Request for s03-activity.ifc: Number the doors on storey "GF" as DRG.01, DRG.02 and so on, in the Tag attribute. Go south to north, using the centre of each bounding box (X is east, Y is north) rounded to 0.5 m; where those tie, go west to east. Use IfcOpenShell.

First a look at what the model holds.

```python
import ifcopenshell
import ifcopenshell.util.element
import ifcopenshell.util.placement

model = ifcopenshell.open("s03-activity.ifc")
print(model.schema)
storey = next(s for s in model.by_type("IfcBuildingStorey") if s.Name == "GF")
doors = [e for e in ifcopenshell.util.element.get_decomposition(storey) if e.is_a("IfcDoor")]
for e in sorted(doors, key=lambda e: e.id()):
    origin = ifcopenshell.util.placement.get_local_placement(e.ObjectPlacement)[:3, 3]
    print(e.id(), e.Tag, e.Name, origin.round(2) + 0.0, sep=" | ")
```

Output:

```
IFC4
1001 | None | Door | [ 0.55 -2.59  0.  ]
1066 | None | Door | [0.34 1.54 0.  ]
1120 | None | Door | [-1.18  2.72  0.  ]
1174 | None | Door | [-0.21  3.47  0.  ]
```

```python
import ifcopenshell
import ifcopenshell.geom
import ifcopenshell.util.element
import ifcopenshell.util.shape

model = ifcopenshell.open("s03-activity.ifc")
settings = ifcopenshell.geom.settings()
settings.set("use-world-coords", True)


def centre(element):
    shape = ifcopenshell.geom.create_shape(settings, element)
    return ifcopenshell.util.shape.get_bbox_centroid(shape.geometry)


storey = next(s for s in model.by_type("IfcBuildingStorey") if s.Name == "GF")
doors = [e for e in ifcopenshell.util.element.get_decomposition(storey) if e.is_a("IfcDoor")]

# Insertion points can sit at a corner or the storey origin, so sort by the geometry (in metres).
centres = {e: centre(e) for e in doors}
doors.sort(key=lambda e: (round(centres[e][1] / 0.5), centres[e][0]))

for i, e in enumerate(doors, start=1):
    number = f"DRG.{i:02d}"
    e.Tag = number
    print(e.id(), number)

model.write("s03-activity_updated.ifc")
```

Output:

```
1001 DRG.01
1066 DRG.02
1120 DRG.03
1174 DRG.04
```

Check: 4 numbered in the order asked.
